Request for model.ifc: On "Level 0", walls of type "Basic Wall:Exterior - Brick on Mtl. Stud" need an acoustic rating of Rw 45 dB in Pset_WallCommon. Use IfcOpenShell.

First a look at what the model holds.

```python
import ifcopenshell
import ifcopenshell.util.element

model = ifcopenshell.open("model.ifc")
print(model.schema)
storey = next(s for s in model.by_type("IfcBuildingStorey") if s.Name == "Level 0")
walls = [e for e in ifcopenshell.util.element.get_decomposition(storey) if e.is_a("IfcWall")]
seen = {}
for e in walls:
    element_type = ifcopenshell.util.element.get_type(e)
    key = (element_type.Name if element_type != e and element_type else None, ifcopenshell.util.element.get_pset(e, "Pset_WallCommon", "AcousticRating"))
    seen[key] = seen.get(key, 0) + 1
for (name, value), count in sorted(seen.items(), key=str):
    print(count, "x", name, "|", value)
```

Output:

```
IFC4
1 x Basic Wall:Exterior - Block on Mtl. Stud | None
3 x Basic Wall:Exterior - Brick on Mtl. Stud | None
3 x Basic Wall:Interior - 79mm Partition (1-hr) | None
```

```python
import ifcopenshell
import ifcopenshell.api.pset
import ifcopenshell.util.element

model = ifcopenshell.open("model.ifc")

storey = next(s for s in model.by_type("IfcBuildingStorey") if s.Name == "Level 0")
walls = [e for e in ifcopenshell.util.element.get_decomposition(storey) if e.is_a("IfcWall")]

count = 0
for e in walls:
    element_type = ifcopenshell.util.element.get_type(e)
    if element_type in (None, e) or element_type.Name != "Basic Wall:Exterior - Brick on Mtl. Stud":
        continue
    # add_pset returns the element's existing set when there is one.
    pset = ifcopenshell.api.pset.add_pset(model, product=e, name="Pset_WallCommon")
    ifcopenshell.api.pset.edit_pset(model, pset=pset, properties={"AcousticRating": "Rw 45 dB"})
    count += 1

print(count, "walls updated")

model.write("model_v2.ifc")
```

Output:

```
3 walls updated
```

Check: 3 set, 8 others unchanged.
